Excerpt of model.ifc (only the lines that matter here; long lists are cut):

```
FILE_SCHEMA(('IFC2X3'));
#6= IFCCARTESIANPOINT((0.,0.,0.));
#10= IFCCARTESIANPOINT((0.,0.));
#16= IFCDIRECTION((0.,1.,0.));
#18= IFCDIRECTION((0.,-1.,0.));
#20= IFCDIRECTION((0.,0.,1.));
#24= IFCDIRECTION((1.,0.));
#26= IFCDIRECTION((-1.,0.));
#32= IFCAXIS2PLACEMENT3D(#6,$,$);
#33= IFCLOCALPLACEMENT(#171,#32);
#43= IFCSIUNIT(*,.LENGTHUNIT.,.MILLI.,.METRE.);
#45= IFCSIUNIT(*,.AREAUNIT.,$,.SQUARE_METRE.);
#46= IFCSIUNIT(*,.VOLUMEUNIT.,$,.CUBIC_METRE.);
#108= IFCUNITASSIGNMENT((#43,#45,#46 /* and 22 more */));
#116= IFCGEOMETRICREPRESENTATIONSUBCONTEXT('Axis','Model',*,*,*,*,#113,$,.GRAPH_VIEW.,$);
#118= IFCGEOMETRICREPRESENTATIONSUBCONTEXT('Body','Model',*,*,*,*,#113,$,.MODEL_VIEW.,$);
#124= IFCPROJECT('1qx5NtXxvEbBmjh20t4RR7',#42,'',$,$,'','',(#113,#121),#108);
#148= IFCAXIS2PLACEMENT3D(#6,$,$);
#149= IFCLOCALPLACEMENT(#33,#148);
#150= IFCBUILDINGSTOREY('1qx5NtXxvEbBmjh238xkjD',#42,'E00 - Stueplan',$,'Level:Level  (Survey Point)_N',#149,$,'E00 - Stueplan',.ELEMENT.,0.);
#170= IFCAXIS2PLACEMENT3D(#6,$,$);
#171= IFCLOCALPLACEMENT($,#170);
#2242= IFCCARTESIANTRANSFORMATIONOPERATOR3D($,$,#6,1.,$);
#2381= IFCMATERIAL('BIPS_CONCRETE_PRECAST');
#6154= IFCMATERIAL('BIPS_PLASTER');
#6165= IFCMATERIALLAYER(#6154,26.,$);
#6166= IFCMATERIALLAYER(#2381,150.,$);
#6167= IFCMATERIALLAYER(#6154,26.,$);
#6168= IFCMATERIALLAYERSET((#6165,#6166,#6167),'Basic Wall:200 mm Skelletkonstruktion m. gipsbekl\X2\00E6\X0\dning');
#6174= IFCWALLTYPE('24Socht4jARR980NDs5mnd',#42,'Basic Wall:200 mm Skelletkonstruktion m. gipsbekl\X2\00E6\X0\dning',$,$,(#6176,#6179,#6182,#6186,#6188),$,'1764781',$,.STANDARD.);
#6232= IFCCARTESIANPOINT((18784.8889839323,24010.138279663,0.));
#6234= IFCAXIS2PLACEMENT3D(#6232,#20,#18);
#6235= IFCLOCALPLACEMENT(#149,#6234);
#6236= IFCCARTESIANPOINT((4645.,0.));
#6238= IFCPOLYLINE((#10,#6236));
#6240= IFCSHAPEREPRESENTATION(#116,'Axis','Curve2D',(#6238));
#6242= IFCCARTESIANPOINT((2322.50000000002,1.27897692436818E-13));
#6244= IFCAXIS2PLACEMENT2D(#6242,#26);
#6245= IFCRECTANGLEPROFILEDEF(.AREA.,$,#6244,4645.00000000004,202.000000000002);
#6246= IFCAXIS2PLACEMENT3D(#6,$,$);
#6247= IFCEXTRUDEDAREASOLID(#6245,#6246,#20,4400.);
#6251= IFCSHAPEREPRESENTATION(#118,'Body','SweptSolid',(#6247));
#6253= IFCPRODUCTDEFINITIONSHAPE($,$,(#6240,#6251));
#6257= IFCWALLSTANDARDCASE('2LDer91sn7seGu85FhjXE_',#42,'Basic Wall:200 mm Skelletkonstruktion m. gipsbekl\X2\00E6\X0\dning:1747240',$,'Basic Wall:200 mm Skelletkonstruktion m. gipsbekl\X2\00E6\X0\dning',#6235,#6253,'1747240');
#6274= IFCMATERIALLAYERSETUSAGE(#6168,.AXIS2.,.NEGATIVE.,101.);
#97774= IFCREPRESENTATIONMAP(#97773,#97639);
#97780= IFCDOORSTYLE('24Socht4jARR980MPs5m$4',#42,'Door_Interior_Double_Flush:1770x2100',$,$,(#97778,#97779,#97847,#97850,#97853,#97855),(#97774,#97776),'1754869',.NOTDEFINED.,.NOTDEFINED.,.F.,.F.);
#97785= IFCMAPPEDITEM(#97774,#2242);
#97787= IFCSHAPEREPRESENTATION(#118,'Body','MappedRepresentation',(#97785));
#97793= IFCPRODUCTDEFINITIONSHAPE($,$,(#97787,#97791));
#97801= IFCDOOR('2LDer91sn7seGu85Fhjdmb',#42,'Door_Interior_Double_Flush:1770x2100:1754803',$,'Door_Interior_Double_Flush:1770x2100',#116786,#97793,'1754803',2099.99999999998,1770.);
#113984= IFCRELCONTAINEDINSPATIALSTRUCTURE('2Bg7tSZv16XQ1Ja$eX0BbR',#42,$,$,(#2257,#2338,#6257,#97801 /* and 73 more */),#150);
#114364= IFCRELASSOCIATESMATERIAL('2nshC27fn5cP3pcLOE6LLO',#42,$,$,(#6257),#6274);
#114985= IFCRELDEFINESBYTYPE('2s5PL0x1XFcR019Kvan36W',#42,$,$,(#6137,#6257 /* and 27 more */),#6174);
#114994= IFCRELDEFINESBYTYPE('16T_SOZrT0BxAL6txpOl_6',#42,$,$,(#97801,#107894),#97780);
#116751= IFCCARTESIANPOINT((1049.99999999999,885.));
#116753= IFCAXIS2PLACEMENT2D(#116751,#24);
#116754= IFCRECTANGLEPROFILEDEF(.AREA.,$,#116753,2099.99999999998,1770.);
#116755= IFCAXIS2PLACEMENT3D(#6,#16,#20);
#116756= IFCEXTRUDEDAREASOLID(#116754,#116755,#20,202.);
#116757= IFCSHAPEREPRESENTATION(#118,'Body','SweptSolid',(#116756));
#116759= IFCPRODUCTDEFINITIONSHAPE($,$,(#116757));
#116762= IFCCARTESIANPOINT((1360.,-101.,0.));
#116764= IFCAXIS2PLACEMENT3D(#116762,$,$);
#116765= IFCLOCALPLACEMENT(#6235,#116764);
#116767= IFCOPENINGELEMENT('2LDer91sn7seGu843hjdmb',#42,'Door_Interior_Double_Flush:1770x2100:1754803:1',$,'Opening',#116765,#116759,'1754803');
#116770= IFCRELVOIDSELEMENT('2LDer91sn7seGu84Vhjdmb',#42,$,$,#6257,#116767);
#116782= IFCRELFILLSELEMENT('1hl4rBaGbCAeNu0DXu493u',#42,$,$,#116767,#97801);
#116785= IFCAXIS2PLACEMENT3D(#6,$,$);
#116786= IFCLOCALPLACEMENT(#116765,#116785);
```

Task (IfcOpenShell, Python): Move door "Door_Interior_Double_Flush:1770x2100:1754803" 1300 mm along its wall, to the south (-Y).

```python
import ifcopenshell
import ifcopenshell.api.geometry
import ifcopenshell.util.placement
import ifcopenshell.util.unit

model = ifcopenshell.open("model.ifc")
unit_scale = ifcopenshell.util.unit.calculate_unit_scale(model)

door = model.by_id(97801)
opening = door.FillsVoids[0].RelatingOpeningElement
wall = opening.VoidsElements[0].RelatingBuildingElement

wall_matrix = ifcopenshell.util.placement.get_local_placement(wall.ObjectPlacement)
shift = wall_matrix[:3, 0] * 1.3 / unit_scale
before = ifcopenshell.util.placement.get_local_placement(door.ObjectPlacement)[:3, 3].copy()

# The door is placed relative to its opening, so it follows when the opening moves.
matrix = ifcopenshell.util.placement.get_local_placement(opening.ObjectPlacement)
matrix[:3, 3] += shift
ifcopenshell.api.geometry.edit_object_placement(
    model, product=opening, matrix=matrix, is_si=False, should_transform_children=True
)

after = ifcopenshell.util.placement.get_local_placement(door.ObjectPlacement)[:3, 3]
print("door moved by", (after - before).round(3) + 0.0)

model.write("model_rev.ifc")
```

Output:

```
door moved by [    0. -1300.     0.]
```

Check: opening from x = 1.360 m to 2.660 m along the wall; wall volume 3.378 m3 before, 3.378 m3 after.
